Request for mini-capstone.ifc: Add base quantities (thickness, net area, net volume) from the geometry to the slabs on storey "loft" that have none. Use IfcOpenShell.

First a look at what the model holds.

```python
import ifcopenshell
import ifcopenshell.util.element
import ifcopenshell.util.unit

model = ifcopenshell.open("mini-capstone.ifc")
print(model.schema)
for unit_type in ("LENGTHUNIT", "AREAUNIT", "VOLUMEUNIT"):
    print(unit_type, ifcopenshell.util.unit.calculate_unit_scale(model, unit_type))
storey = next(s for s in model.by_type("IfcBuildingStorey") if s.Name == "loft")
slabs = [e for e in ifcopenshell.util.element.get_decomposition(storey) if e.is_a("IfcSlab")]
for e in sorted(slabs, key=lambda e: e.id()):
    print(e.id(), e.is_a(), e.Name, list(ifcopenshell.util.element.get_psets(e, qtos_only=True)), sep=" | ")
```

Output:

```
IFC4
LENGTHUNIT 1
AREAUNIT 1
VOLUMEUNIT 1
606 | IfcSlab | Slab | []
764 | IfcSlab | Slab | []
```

```python
import ifcopenshell
import ifcopenshell.api.pset
import ifcopenshell.geom
import ifcopenshell.util.element
import ifcopenshell.util.shape
import ifcopenshell.util.unit

model = ifcopenshell.open("mini-capstone.ifc")
unit_scale = ifcopenshell.util.unit.calculate_unit_scale(model)
area_scale = ifcopenshell.util.unit.calculate_unit_scale(model, "AREAUNIT")
volume_scale = ifcopenshell.util.unit.calculate_unit_scale(model, "VOLUMEUNIT")
settings = ifcopenshell.geom.settings()

storey = next(s for s in model.by_type("IfcBuildingStorey") if s.Name == "loft")
slabs = [e for e in ifcopenshell.util.element.get_decomposition(storey) if e.is_a("IfcSlab")]

for e in sorted(slabs, key=lambda e: e.id()):
    if ifcopenshell.util.element.get_psets(e, qtos_only=True, should_inherit=False):
        continue
    # Geometry comes back in metres, in the element's own axes.
    shape = ifcopenshell.geom.create_shape(settings, e)
    values = {
        "Width": ifcopenshell.util.shape.get_z(shape.geometry) / unit_scale,
        "NetArea": ifcopenshell.util.shape.get_footprint_area(shape.geometry) / area_scale,
        "NetVolume": ifcopenshell.util.shape.get_volume(shape.geometry) / volume_scale,
    }
    qto = ifcopenshell.api.pset.add_qto(model, product=e, name="Qto_SlabBaseQuantities")
    ifcopenshell.api.pset.edit_qto(model, qto=qto, properties=values)
    print(e.id(), {k: round(v, 3) for k, v in values.items()})

model.write("mini-capstone_rev.ifc")
```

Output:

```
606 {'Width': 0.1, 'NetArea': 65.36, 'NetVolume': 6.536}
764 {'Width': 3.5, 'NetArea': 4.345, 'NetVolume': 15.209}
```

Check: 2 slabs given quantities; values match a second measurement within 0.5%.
